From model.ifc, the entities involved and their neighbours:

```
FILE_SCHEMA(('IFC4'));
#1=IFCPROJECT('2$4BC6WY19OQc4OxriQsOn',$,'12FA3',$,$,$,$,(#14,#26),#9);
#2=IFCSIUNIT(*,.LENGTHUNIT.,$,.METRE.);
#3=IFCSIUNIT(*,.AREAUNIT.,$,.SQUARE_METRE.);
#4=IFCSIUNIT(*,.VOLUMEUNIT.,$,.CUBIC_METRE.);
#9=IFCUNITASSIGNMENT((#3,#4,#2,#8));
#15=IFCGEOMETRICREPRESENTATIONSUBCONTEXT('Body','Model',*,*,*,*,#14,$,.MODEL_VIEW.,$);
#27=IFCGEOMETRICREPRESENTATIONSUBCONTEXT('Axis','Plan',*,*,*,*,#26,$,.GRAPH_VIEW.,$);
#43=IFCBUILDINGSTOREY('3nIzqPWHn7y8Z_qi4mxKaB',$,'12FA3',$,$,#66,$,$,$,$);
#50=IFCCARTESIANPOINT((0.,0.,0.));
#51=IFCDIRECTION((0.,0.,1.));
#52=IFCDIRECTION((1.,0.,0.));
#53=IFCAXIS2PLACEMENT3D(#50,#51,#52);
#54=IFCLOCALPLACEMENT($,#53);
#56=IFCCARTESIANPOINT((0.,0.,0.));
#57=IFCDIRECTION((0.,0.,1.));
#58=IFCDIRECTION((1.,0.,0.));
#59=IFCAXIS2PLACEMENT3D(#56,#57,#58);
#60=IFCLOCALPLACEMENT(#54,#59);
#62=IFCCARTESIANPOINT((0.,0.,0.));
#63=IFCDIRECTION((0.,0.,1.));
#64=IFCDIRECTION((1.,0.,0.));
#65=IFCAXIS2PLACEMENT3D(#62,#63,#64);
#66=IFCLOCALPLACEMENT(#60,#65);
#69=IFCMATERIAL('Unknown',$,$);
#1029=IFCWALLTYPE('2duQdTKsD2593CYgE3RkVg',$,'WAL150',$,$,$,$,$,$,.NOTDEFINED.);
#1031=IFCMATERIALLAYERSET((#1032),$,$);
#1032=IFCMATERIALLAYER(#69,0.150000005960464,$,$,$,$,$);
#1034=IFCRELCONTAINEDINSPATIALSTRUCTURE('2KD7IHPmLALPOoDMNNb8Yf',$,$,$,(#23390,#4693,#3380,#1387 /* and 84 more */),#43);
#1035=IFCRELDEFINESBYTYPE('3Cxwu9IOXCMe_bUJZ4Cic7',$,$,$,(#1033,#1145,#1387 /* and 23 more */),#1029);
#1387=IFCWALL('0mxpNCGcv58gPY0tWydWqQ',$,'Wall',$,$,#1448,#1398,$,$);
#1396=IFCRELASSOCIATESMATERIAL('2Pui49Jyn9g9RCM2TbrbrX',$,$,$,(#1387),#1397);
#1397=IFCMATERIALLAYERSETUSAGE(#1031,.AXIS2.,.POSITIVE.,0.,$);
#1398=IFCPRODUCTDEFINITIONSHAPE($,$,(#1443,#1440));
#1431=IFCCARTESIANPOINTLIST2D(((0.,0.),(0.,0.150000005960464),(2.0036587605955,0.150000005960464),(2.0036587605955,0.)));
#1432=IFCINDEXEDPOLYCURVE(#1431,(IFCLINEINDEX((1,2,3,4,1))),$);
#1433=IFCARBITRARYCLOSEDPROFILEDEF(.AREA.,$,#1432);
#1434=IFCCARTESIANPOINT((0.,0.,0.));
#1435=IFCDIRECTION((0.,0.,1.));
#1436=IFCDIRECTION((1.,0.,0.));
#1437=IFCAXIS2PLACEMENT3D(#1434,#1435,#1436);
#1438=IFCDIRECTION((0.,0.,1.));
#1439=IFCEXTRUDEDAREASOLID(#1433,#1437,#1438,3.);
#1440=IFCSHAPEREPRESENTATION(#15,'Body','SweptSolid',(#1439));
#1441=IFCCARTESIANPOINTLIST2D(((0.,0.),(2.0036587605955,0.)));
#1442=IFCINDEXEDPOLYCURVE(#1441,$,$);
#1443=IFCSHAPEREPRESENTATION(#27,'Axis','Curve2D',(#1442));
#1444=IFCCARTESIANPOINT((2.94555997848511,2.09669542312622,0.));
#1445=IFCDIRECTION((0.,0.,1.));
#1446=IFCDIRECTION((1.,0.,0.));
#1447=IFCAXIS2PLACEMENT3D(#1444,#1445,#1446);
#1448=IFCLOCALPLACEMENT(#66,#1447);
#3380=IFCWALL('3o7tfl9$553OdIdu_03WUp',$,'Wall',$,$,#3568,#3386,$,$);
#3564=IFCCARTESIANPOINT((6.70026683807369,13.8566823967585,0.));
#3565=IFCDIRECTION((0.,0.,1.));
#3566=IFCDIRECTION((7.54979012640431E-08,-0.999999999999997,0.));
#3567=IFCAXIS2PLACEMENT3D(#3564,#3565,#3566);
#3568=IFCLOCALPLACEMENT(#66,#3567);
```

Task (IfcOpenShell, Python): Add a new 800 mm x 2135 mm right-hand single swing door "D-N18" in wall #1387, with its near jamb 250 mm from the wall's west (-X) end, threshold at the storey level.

```python
import numpy as np
import ifcopenshell
import ifcopenshell.api.feature
import ifcopenshell.api.geometry
import ifcopenshell.api.root
import ifcopenshell.api.spatial
import ifcopenshell.geom
import ifcopenshell.util.element
import ifcopenshell.util.placement
import ifcopenshell.util.representation
import ifcopenshell.util.shape
import ifcopenshell.util.unit

model = ifcopenshell.open("model.ifc")
unit_scale = ifcopenshell.util.unit.calculate_unit_scale(model)
settings = ifcopenshell.geom.settings()


def volume(element):
    """Net volume in cubic metres, openings subtracted."""
    shape = ifcopenshell.geom.create_shape(settings, element)
    return ifcopenshell.util.shape.get_volume(shape.geometry)


wall = model.by_guid("0mxpNCGcv58gPY0tWydWqQ")
storey = ifcopenshell.util.element.get_container(wall, ifc_class="IfcBuildingStorey")
context = ifcopenshell.util.representation.get_context(model, "Model", "Body", "MODEL_VIEW")
before = volume(wall)

width, height, from_end, sill = 0.8, 2.135, 0.25, 0.0  # metres

# The wall runs along its own X axis, and the end named is its -X end.
wall_shape = ifcopenshell.geom.create_shape(settings, wall)
x, y, z = ifcopenshell.util.shape.get_vertices(wall_shape.geometry).T
start = x.min() + from_end
face, thickness = float(y.min()), float(y.max() - y.min())
wall_matrix = ifcopenshell.util.placement.get_local_placement(wall.ObjectPlacement)
level = ifcopenshell.util.placement.get_local_placement(storey.ObjectPlacement)[2, 3]


def in_wall(x, y):
    """Placement at x, y metres in the wall's axes, at sill height."""
    matrix = wall_matrix.copy()
    matrix[:, 3] = wall_matrix @ np.array([x / unit_scale, y / unit_scale, 0.0, 1.0])
    matrix[2, 3] = level + sill / unit_scale
    return matrix


# Opening: a box that overshoots both wall faces by 50 mm.
opening = ifcopenshell.api.root.create_entity(model, ifc_class="IfcOpeningElement", predefined_type="OPENING")
box = ifcopenshell.api.geometry.add_wall_representation(
    model, context=context, length=width, height=height, thickness=thickness + 0.1
)
ifcopenshell.api.geometry.assign_representation(model, product=opening, representation=box)
ifcopenshell.api.geometry.edit_object_placement(model, product=opening, matrix=in_wall(start, face - 0.05), is_si=False)
ifcopenshell.api.feature.add_feature(model, feature=opening, element=wall)

door = ifcopenshell.api.root.create_entity(model, ifc_class="IfcDoor", name="D-N18", predefined_type="DOOR")
door.OverallWidth, door.OverallHeight = width / unit_scale, height / unit_scale
door.OperationType = "SINGLE_SWING_RIGHT"
body = ifcopenshell.api.geometry.add_door_representation(
    model,
    context=context,
    overall_width=door.OverallWidth,
    overall_height=door.OverallHeight,
    operation_type="SINGLE_SWING_RIGHT",
    lining_properties={"LiningDepth": thickness / unit_scale, "ThresholdDepth": thickness / unit_scale},
)
ifcopenshell.api.geometry.assign_representation(model, product=door, representation=body)
ifcopenshell.api.spatial.assign_container(model, products=[door], relating_structure=storey)
ifcopenshell.api.feature.add_filling(model, opening=opening, element=door)

# The lining spans the wall, so the door starts at the wall face.
ifcopenshell.api.geometry.edit_object_placement(model, product=door, matrix=in_wall(start, face), is_si=False)

after = volume(wall)

print(f"wall volume {before:.3f} -> {after:.3f} m3")

model.write("model_edited.ifc")
```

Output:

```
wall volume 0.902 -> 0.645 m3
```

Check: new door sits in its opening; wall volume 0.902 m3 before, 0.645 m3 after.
